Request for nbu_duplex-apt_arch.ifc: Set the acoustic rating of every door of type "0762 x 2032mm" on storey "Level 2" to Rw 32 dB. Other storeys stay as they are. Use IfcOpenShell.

First a look at what the model holds.

```python
import ifcopenshell
import ifcopenshell.util.element

model = ifcopenshell.open("nbu_duplex-apt_arch.ifc")
print(model.schema)
storey = next(s for s in model.by_type("IfcBuildingStorey") if s.Name == "Level 2")
doors = [e for e in ifcopenshell.util.element.get_decomposition(storey) if e.is_a("IfcDoor")]
seen = {}
for e in doors:
    element_type = ifcopenshell.util.element.get_type(e)
    key = (element_type.Name if element_type != e and element_type else None, ifcopenshell.util.element.get_pset(e, "Pset_DoorCommon", "AcousticRating"))
    seen[key] = seen.get(key, 0) + 1
for (name, value), count in sorted(seen.items(), key=str):
    print(count, "x", name, "|", value)
```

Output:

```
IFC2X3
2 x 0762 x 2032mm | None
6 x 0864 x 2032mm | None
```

```python
import ifcopenshell
import ifcopenshell.api.pset
import ifcopenshell.util.element

model = ifcopenshell.open("nbu_duplex-apt_arch.ifc")

storey = next(s for s in model.by_type("IfcBuildingStorey") if s.Name == "Level 2")
doors = [e for e in ifcopenshell.util.element.get_decomposition(storey) if e.is_a("IfcDoor")]

count = 0
for e in doors:
    element_type = ifcopenshell.util.element.get_type(e)
    if element_type in (None, e) or element_type.Name != "0762 x 2032mm":
        continue
    # add_pset returns the element's existing set when there is one.
    pset = ifcopenshell.api.pset.add_pset(model, product=e, name="Pset_DoorCommon")
    ifcopenshell.api.pset.edit_pset(model, pset=pset, properties={"AcousticRating": "Rw 32 dB"})
    count += 1

print(count, "doors updated")

model.write("nbu_duplex-apt_arch_rev.ifc")
```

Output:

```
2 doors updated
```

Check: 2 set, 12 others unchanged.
